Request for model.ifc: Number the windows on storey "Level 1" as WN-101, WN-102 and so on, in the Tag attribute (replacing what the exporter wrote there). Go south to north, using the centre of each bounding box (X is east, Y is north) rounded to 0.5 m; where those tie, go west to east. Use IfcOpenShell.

First a look at what the model holds.

```python
import ifcopenshell
import ifcopenshell.util.element
import ifcopenshell.util.placement

model = ifcopenshell.open("model.ifc")
print(model.schema)
storey = next(s for s in model.by_type("IfcBuildingStorey") if s.Name == "Level 1")
windows = [e for e in ifcopenshell.util.element.get_decomposition(storey) if e.is_a("IfcWindow")]
for e in sorted(windows, key=lambda e: e.id()):
    origin = ifcopenshell.util.placement.get_local_placement(e.ObjectPlacement)[:3, 3]
    print(e.id(), e.Tag, e.Name, origin.round(2) + 0.0, sep=" | ")
```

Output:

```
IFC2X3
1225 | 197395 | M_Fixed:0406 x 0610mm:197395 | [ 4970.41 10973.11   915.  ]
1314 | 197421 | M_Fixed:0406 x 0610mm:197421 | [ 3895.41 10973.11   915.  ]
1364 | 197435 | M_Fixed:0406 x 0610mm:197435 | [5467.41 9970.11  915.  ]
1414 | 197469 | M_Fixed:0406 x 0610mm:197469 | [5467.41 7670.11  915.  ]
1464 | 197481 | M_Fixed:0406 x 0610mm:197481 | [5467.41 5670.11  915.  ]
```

```python
import ifcopenshell
import ifcopenshell.geom
import ifcopenshell.util.element
import ifcopenshell.util.shape

model = ifcopenshell.open("model.ifc")
settings = ifcopenshell.geom.settings()
settings.set("use-world-coords", True)


def centre(element):
    shape = ifcopenshell.geom.create_shape(settings, element)
    return ifcopenshell.util.shape.get_bbox_centroid(shape.geometry)


storey = next(s for s in model.by_type("IfcBuildingStorey") if s.Name == "Level 1")
windows = [e for e in ifcopenshell.util.element.get_decomposition(storey) if e.is_a("IfcWindow")]

# Insertion points can sit at a corner or the storey origin, so sort by the geometry (in metres).
centres = {e: centre(e) for e in windows}
windows.sort(key=lambda e: (round(centres[e][1] / 0.5), centres[e][0]))

for i, e in enumerate(windows, start=1):
    number = f"WN-1{i:02d}"
    e.Tag = number
    print(e.id(), number)

model.write("model-out.ifc")
```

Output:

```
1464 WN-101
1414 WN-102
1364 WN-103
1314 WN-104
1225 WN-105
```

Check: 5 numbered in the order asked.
